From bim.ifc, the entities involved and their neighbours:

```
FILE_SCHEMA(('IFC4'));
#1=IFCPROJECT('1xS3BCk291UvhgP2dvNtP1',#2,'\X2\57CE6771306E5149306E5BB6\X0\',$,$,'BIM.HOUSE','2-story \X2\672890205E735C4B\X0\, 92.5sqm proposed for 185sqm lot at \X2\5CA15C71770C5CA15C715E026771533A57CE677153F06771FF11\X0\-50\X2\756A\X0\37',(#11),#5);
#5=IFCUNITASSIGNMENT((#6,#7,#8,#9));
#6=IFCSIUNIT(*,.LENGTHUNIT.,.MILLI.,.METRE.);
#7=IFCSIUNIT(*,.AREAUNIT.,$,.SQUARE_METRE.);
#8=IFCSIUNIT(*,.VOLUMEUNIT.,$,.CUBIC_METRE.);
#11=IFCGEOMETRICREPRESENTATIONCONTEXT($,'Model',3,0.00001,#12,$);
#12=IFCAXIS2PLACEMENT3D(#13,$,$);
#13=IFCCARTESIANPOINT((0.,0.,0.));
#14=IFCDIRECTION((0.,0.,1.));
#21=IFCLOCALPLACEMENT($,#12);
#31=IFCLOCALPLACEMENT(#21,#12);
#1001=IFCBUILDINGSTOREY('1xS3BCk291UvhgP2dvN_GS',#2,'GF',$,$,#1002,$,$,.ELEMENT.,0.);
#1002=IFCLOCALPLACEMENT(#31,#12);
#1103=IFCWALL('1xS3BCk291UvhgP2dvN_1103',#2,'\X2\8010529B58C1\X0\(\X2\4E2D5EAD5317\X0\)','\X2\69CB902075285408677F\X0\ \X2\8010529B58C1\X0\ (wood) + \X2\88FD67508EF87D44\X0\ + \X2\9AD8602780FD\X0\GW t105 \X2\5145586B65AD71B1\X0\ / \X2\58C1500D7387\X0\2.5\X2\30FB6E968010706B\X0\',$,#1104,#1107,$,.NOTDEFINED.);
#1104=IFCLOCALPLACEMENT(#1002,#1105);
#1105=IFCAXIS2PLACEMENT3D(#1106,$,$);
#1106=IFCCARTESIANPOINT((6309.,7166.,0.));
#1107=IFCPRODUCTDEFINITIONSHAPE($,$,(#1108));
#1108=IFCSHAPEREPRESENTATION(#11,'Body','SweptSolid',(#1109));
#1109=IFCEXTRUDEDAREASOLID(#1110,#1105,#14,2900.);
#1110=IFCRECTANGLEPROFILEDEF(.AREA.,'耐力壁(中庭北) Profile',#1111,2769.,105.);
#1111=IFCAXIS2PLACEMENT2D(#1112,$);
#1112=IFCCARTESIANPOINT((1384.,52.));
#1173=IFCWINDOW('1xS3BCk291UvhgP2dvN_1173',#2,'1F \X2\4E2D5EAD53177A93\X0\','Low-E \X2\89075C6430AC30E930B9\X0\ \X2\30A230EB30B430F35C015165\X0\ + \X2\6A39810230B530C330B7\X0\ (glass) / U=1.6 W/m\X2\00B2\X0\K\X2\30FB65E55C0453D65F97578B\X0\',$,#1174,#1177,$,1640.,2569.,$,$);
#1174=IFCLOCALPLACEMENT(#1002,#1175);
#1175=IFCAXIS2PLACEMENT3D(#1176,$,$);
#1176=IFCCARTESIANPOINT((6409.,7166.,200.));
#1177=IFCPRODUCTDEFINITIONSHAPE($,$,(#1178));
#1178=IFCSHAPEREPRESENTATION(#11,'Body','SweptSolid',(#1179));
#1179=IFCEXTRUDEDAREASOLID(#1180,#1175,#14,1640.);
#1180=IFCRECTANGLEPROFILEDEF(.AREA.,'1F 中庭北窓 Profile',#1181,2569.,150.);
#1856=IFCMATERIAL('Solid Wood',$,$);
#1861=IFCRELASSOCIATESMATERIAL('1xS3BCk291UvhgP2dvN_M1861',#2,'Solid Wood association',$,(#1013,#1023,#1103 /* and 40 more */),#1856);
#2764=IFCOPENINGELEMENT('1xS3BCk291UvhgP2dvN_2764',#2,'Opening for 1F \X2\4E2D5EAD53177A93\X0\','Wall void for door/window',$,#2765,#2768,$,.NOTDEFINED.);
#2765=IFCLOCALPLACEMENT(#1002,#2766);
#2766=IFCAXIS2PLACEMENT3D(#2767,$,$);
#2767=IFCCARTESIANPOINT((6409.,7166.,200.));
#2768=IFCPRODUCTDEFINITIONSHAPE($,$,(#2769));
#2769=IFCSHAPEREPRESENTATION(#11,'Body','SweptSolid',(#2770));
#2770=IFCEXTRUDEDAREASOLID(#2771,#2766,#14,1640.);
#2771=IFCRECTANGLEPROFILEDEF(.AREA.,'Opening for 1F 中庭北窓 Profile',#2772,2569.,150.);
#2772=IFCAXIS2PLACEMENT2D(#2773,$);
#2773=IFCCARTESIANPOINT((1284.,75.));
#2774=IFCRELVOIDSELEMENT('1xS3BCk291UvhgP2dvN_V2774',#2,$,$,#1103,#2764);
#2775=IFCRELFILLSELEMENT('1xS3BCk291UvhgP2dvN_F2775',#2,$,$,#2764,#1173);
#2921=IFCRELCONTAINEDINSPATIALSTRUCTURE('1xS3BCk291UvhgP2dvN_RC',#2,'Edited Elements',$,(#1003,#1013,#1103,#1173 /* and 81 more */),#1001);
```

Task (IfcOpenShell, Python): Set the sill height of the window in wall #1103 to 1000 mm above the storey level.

```python
import numpy as np
import ifcopenshell
import ifcopenshell.api.geometry
import ifcopenshell.geom
import ifcopenshell.util.element
import ifcopenshell.util.placement
import ifcopenshell.util.shape
import ifcopenshell.util.unit

model = ifcopenshell.open("bim.ifc")
unit_scale = ifcopenshell.util.unit.calculate_unit_scale(model)

window = model.by_id(1173)
opening = window.FillsVoids[0].RelatingOpeningElement
storey = ifcopenshell.util.element.get_container(window, ifc_class="IfcBuildingStorey")
level = ifcopenshell.util.placement.get_local_placement(storey.ObjectPlacement)[2, 3]

# The opening's origin need not be at the sill, so measure its lowest point.
shape = ifcopenshell.geom.create_shape(ifcopenshell.geom.settings(), opening)
bottom = ifcopenshell.util.shape.get_shape_bottom_elevation(shape, shape.geometry) / unit_scale
dz = level + 1000.0 - bottom

shift = np.array([0.0, 0.0, dz])
# The window is not placed relative to its opening, so move both.
for product in (opening, window):
    matrix = ifcopenshell.util.placement.get_local_placement(product.ObjectPlacement)
    matrix[:3, 3] += shift
    ifcopenshell.api.geometry.edit_object_placement(model, product=product, matrix=matrix, is_si=False)

print(f"moved by {dz * unit_scale:+.3f} m")

model.write("bim_rev.ifc")
```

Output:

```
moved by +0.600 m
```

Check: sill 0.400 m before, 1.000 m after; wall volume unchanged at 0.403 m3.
